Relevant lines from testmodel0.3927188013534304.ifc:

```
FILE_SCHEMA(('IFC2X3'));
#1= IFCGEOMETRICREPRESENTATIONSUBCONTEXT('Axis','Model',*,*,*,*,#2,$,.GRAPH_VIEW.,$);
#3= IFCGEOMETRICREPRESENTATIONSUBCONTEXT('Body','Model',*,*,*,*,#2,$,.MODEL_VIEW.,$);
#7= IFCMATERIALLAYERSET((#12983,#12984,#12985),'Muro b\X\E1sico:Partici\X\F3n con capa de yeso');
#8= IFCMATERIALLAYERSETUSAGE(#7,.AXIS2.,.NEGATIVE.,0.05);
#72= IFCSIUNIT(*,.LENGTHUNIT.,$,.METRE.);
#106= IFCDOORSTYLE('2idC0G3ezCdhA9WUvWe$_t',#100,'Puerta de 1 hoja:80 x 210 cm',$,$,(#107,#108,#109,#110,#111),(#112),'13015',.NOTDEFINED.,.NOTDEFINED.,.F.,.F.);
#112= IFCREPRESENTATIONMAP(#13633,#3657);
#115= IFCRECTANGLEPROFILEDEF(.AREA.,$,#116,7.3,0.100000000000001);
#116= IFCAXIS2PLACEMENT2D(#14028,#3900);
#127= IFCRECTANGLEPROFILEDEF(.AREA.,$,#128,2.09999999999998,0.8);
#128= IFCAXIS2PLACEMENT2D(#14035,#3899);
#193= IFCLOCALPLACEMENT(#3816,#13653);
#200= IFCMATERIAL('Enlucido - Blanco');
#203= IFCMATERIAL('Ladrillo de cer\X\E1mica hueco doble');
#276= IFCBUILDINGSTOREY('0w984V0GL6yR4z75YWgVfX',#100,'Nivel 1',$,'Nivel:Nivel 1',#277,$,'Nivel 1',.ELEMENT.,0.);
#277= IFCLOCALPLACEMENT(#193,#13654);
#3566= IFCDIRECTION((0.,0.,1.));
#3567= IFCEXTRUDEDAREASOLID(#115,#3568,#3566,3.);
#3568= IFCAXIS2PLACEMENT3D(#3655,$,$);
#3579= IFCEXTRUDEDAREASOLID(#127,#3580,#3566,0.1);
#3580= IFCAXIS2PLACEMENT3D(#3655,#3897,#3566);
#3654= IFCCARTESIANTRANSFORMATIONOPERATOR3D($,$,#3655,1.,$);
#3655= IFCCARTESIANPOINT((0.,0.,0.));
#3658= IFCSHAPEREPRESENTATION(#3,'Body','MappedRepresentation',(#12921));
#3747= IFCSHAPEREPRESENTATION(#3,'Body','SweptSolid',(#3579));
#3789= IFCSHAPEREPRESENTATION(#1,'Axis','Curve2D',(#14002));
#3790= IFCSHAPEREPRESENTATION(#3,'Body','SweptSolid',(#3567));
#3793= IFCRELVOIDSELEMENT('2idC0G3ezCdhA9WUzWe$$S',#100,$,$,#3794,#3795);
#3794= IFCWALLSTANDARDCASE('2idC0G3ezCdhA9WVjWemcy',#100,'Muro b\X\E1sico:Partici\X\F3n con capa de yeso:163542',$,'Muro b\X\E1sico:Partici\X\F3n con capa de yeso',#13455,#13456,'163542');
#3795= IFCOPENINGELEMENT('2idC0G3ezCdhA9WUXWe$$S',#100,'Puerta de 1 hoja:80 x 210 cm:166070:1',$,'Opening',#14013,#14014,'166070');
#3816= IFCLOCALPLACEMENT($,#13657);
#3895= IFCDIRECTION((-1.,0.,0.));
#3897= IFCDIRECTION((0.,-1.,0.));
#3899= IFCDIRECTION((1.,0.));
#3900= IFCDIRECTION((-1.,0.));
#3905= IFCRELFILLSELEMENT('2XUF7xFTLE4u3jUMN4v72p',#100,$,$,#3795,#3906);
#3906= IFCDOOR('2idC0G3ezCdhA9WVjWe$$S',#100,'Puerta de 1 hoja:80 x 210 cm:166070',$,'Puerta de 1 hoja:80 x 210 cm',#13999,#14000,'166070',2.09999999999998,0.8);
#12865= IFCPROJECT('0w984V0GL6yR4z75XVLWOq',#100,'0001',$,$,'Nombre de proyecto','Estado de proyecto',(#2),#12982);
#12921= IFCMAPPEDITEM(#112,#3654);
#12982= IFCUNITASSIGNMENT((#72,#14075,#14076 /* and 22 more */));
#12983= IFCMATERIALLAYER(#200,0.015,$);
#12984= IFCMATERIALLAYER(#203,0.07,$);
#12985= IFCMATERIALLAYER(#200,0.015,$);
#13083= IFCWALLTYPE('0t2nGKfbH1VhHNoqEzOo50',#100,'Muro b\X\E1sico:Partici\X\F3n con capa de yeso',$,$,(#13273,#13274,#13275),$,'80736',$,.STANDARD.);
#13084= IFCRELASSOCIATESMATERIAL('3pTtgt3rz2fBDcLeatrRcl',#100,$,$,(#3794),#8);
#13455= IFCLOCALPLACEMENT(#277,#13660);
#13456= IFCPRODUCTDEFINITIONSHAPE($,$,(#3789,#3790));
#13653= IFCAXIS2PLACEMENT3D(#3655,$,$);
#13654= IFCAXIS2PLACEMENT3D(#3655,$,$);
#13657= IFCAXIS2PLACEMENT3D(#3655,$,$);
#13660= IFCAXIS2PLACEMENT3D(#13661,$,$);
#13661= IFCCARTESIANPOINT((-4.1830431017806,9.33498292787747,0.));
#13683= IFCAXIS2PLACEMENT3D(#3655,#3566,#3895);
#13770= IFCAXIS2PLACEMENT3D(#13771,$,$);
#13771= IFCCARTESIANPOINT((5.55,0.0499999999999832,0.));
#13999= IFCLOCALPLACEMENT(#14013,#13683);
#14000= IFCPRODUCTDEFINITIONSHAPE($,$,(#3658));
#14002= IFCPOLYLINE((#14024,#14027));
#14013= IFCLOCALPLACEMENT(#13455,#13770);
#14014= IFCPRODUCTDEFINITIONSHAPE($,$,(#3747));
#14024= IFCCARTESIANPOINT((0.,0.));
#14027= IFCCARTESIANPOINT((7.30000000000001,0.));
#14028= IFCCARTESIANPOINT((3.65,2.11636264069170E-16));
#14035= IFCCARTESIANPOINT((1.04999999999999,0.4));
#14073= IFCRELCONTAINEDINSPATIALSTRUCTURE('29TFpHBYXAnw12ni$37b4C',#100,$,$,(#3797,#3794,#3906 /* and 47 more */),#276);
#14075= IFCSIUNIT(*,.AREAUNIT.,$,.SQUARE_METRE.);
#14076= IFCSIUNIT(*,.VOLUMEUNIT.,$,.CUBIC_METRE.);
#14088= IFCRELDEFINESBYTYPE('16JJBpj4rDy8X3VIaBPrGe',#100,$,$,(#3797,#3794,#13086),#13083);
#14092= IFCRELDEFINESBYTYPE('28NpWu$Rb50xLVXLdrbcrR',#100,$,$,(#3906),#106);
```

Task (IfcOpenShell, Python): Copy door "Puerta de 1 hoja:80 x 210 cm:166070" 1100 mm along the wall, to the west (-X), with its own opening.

```python
import ifcopenshell
import ifcopenshell.api.feature
import ifcopenshell.api.geometry
import ifcopenshell.api.root
import ifcopenshell.geom
import ifcopenshell.util.element
import ifcopenshell.util.placement
import ifcopenshell.util.shape
import ifcopenshell.util.unit

model = ifcopenshell.open("testmodel0.3927188013534304.ifc")
unit_scale = ifcopenshell.util.unit.calculate_unit_scale(model)
settings = ifcopenshell.geom.settings()


def volume(element):
    """Net volume in cubic metres, openings subtracted."""
    shape = ifcopenshell.geom.create_shape(settings, element)
    return ifcopenshell.util.shape.get_volume(shape.geometry)


def reuse_history(source, copy):
    """copy_class also copies each property set's owner history, people and application; keep the originals."""
    for rel in copy.IsDefinedBy:
        if rel.is_a("IfcRelDefinesByProperties") and (history := rel.RelatingPropertyDefinition.OwnerHistory):
            rel.RelatingPropertyDefinition.OwnerHistory = source.OwnerHistory
            ifcopenshell.util.element.remove_deep2(model, history)


door = model.by_guid("2idC0G3ezCdhA9WVjWe$$S")
opening = door.FillsVoids[0].RelatingOpeningElement
wall = opening.VoidsElements[0].RelatingBuildingElement
before = volume(wall)
shift = ifcopenshell.util.placement.get_local_placement(wall.ObjectPlacement)[:3, 0] * -1.1 / unit_scale

# copy_class copies the void relationship, type, container and properties, but no geometry.
new_opening = ifcopenshell.api.root.copy_class(model, product=opening)
new_opening.Representation = ifcopenshell.util.element.copy_deep(
    model, opening.Representation, exclude=["IfcGeometricRepresentationContext", "IfcRepresentationMap"]
)
new_opening.Name = "Puerta de 1 hoja:80 x 210 cm"
new_opening.Tag = None
new_door = ifcopenshell.api.root.copy_class(model, product=door)
new_door.Representation = ifcopenshell.util.element.copy_deep(
    model, door.Representation, exclude=["IfcGeometricRepresentationContext", "IfcRepresentationMap"]
)
new_door.Name = "Puerta de 1 hoja:80 x 210 cm"
new_door.Tag = None
reuse_history(door, new_door)
fills = ifcopenshell.api.feature.add_filling(model, opening=new_opening, element=new_door)
fills.OwnerHistory = new_door.OwnerHistory  # required in IFC2X3

for old, new in ((opening, new_opening), (door, new_door)):
    matrix = ifcopenshell.util.placement.get_local_placement(old.ObjectPlacement)
    matrix[:3, 3] += shift
    ifcopenshell.api.geometry.edit_object_placement(model, product=new, matrix=matrix, is_si=False)

after = volume(wall)

print(f"wall volume {before:.3f} -> {after:.3f} m3")

model.write("testmodel0.3927188013534304_v2.ifc")
```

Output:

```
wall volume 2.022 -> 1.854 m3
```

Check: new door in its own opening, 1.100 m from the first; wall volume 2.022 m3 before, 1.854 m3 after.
